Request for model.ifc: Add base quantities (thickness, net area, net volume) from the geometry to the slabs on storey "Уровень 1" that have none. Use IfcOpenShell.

First a look at what the model holds.

```python
import ifcopenshell
import ifcopenshell.util.element
import ifcopenshell.util.unit

model = ifcopenshell.open("model.ifc")
print(model.schema)
for unit_type in ("LENGTHUNIT", "AREAUNIT", "VOLUMEUNIT"):
    print(unit_type, ifcopenshell.util.unit.calculate_unit_scale(model, unit_type))
storey = next(s for s in model.by_type("IfcBuildingStorey") if s.Name == "Уровень 1")
slabs = [e for e in ifcopenshell.util.element.get_decomposition(storey) if e.is_a("IfcSlab")]
for e in sorted(slabs, key=lambda e: e.id()):
    print(e.id(), e.is_a(), e.Name, list(ifcopenshell.util.element.get_psets(e, qtos_only=True)), sep=" | ")
```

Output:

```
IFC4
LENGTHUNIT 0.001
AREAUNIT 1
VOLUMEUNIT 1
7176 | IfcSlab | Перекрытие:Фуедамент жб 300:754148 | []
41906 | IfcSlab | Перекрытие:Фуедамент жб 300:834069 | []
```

```python
import ifcopenshell
import ifcopenshell.api.pset
import ifcopenshell.geom
import ifcopenshell.util.element
import ifcopenshell.util.shape
import ifcopenshell.util.unit

model = ifcopenshell.open("model.ifc")
unit_scale = ifcopenshell.util.unit.calculate_unit_scale(model)
area_scale = ifcopenshell.util.unit.calculate_unit_scale(model, "AREAUNIT")
volume_scale = ifcopenshell.util.unit.calculate_unit_scale(model, "VOLUMEUNIT")
settings = ifcopenshell.geom.settings()

storey = next(s for s in model.by_type("IfcBuildingStorey") if s.Name == "Уровень 1")
slabs = [e for e in ifcopenshell.util.element.get_decomposition(storey) if e.is_a("IfcSlab")]

for e in sorted(slabs, key=lambda e: e.id()):
    if ifcopenshell.util.element.get_psets(e, qtos_only=True, should_inherit=False):
        continue
    # Geometry comes back in metres, in the element's own axes.
    shape = ifcopenshell.geom.create_shape(settings, e)
    values = {
        "Width": ifcopenshell.util.shape.get_z(shape.geometry) / unit_scale,
        "NetArea": ifcopenshell.util.shape.get_footprint_area(shape.geometry) / area_scale,
        "NetVolume": ifcopenshell.util.shape.get_volume(shape.geometry) / volume_scale,
    }
    qto = ifcopenshell.api.pset.add_qto(model, product=e, name="Qto_SlabBaseQuantities")
    ifcopenshell.api.pset.edit_qto(model, qto=qto, properties=values)
    print(e.id(), {k: round(v, 3) for k, v in values.items()})

model.write("model_updated.ifc")
```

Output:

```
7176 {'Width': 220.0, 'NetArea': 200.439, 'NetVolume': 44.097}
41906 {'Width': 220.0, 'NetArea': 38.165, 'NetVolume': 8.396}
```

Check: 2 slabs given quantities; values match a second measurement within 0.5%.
